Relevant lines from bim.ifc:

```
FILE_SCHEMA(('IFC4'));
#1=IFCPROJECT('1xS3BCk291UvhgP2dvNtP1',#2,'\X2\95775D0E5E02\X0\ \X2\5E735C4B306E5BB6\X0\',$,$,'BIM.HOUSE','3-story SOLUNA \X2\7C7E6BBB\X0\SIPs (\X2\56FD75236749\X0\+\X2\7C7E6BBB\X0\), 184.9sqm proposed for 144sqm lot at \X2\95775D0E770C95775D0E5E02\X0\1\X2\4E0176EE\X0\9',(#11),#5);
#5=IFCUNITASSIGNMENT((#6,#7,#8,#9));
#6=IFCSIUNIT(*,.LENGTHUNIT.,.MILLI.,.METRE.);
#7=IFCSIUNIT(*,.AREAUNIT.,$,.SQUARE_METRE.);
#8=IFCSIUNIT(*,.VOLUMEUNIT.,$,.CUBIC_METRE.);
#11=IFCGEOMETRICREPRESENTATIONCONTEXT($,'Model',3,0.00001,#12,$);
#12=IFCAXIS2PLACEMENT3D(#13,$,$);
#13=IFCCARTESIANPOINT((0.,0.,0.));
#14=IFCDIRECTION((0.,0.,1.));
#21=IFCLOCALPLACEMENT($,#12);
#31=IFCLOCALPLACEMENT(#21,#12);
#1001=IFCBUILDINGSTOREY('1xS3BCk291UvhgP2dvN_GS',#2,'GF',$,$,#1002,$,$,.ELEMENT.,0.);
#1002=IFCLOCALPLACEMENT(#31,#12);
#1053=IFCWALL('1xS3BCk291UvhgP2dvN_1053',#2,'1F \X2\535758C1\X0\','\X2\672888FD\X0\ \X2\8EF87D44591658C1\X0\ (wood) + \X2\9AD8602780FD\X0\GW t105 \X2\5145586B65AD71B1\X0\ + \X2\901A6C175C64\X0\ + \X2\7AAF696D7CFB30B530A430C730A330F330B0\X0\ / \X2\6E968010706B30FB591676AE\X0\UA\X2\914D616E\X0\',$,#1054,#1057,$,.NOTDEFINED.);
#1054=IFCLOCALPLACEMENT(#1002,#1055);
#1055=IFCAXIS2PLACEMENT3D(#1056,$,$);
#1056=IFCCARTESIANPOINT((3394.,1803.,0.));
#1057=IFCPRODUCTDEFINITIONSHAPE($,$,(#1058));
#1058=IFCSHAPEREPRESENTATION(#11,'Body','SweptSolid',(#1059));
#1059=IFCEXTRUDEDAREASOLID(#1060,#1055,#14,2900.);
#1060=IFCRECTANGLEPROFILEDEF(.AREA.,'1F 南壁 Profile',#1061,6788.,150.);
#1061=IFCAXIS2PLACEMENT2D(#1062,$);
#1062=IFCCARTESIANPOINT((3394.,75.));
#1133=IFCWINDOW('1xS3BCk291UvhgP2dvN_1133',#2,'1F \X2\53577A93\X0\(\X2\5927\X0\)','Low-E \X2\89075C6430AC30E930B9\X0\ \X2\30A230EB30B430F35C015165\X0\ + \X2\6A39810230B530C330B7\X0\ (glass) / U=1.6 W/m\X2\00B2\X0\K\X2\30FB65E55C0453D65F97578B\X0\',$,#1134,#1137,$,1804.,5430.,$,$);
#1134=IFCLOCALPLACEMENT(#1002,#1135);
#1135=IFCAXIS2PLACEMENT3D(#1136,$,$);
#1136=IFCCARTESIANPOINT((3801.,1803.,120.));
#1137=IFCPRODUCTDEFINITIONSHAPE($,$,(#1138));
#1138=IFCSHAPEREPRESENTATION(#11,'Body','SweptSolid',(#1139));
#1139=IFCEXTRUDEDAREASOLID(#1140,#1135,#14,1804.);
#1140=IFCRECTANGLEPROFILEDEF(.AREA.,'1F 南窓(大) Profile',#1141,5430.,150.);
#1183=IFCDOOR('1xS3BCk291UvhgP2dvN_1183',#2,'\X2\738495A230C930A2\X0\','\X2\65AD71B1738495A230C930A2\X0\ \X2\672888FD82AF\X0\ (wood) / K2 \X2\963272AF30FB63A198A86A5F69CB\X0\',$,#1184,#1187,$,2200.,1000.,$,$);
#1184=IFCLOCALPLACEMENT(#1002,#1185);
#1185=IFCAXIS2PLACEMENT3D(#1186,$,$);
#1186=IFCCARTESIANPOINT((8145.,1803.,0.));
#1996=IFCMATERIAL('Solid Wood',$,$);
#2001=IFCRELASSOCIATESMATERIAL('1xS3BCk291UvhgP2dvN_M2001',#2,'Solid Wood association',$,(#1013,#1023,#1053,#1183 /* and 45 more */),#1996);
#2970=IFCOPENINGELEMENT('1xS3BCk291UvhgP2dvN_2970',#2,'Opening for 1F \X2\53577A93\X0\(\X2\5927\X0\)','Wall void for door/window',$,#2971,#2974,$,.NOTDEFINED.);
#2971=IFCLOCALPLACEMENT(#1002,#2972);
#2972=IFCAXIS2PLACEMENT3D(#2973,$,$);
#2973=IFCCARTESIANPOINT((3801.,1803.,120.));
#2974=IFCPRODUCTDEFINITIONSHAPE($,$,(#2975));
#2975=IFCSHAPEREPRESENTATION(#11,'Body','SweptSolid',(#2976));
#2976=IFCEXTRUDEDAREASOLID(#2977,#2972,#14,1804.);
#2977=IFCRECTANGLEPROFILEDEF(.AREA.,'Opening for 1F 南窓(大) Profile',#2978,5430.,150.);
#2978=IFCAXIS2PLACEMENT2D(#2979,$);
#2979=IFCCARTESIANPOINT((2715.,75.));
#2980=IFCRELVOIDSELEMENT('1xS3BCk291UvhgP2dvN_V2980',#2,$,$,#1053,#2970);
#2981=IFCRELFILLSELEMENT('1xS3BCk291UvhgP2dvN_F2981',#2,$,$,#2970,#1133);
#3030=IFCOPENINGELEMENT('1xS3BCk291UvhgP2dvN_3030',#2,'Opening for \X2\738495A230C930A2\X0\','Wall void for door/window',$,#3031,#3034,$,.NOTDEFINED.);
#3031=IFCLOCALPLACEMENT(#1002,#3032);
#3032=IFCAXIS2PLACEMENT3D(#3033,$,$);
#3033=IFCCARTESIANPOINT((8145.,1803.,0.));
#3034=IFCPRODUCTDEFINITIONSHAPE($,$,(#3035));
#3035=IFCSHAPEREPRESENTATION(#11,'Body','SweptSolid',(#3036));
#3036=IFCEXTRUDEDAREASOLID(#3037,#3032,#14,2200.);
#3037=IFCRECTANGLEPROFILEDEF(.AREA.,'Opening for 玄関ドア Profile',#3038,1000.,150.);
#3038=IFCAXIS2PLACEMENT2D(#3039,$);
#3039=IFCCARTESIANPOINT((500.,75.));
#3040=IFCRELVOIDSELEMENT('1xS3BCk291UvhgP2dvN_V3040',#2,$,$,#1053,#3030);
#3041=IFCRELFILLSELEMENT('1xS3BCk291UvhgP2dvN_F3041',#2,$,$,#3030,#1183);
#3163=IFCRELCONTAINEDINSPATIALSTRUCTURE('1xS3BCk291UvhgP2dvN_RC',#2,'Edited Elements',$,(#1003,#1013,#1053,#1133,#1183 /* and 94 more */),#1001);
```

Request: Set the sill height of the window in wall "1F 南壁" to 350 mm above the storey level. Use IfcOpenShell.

```python
import numpy as np
import ifcopenshell
import ifcopenshell.api.geometry
import ifcopenshell.geom
import ifcopenshell.util.element
import ifcopenshell.util.placement
import ifcopenshell.util.shape
import ifcopenshell.util.unit

model = ifcopenshell.open("bim.ifc")
unit_scale = ifcopenshell.util.unit.calculate_unit_scale(model)

window = model.by_guid("1xS3BCk291UvhgP2dvN_1133")
opening = window.FillsVoids[0].RelatingOpeningElement
storey = ifcopenshell.util.element.get_container(window, ifc_class="IfcBuildingStorey")
level = ifcopenshell.util.placement.get_local_placement(storey.ObjectPlacement)[2, 3]

# The opening's origin need not be at the sill, so measure its lowest point.
shape = ifcopenshell.geom.create_shape(ifcopenshell.geom.settings(), opening)
bottom = ifcopenshell.util.shape.get_shape_bottom_elevation(shape, shape.geometry) / unit_scale
dz = level + 0.35 / unit_scale - bottom

shift = np.array([0.0, 0.0, dz])
# The window is not placed relative to its opening, so move both.
for product in (opening, window):
    matrix = ifcopenshell.util.placement.get_local_placement(product.ObjectPlacement)
    matrix[:3, 3] += shift
    ifcopenshell.api.geometry.edit_object_placement(model, product=product, matrix=matrix, is_si=False)

print(f"moved by {dz * unit_scale:+.3f} m")

model.write("bim_rev.ifc")
```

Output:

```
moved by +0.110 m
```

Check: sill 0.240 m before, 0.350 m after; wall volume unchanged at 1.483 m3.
